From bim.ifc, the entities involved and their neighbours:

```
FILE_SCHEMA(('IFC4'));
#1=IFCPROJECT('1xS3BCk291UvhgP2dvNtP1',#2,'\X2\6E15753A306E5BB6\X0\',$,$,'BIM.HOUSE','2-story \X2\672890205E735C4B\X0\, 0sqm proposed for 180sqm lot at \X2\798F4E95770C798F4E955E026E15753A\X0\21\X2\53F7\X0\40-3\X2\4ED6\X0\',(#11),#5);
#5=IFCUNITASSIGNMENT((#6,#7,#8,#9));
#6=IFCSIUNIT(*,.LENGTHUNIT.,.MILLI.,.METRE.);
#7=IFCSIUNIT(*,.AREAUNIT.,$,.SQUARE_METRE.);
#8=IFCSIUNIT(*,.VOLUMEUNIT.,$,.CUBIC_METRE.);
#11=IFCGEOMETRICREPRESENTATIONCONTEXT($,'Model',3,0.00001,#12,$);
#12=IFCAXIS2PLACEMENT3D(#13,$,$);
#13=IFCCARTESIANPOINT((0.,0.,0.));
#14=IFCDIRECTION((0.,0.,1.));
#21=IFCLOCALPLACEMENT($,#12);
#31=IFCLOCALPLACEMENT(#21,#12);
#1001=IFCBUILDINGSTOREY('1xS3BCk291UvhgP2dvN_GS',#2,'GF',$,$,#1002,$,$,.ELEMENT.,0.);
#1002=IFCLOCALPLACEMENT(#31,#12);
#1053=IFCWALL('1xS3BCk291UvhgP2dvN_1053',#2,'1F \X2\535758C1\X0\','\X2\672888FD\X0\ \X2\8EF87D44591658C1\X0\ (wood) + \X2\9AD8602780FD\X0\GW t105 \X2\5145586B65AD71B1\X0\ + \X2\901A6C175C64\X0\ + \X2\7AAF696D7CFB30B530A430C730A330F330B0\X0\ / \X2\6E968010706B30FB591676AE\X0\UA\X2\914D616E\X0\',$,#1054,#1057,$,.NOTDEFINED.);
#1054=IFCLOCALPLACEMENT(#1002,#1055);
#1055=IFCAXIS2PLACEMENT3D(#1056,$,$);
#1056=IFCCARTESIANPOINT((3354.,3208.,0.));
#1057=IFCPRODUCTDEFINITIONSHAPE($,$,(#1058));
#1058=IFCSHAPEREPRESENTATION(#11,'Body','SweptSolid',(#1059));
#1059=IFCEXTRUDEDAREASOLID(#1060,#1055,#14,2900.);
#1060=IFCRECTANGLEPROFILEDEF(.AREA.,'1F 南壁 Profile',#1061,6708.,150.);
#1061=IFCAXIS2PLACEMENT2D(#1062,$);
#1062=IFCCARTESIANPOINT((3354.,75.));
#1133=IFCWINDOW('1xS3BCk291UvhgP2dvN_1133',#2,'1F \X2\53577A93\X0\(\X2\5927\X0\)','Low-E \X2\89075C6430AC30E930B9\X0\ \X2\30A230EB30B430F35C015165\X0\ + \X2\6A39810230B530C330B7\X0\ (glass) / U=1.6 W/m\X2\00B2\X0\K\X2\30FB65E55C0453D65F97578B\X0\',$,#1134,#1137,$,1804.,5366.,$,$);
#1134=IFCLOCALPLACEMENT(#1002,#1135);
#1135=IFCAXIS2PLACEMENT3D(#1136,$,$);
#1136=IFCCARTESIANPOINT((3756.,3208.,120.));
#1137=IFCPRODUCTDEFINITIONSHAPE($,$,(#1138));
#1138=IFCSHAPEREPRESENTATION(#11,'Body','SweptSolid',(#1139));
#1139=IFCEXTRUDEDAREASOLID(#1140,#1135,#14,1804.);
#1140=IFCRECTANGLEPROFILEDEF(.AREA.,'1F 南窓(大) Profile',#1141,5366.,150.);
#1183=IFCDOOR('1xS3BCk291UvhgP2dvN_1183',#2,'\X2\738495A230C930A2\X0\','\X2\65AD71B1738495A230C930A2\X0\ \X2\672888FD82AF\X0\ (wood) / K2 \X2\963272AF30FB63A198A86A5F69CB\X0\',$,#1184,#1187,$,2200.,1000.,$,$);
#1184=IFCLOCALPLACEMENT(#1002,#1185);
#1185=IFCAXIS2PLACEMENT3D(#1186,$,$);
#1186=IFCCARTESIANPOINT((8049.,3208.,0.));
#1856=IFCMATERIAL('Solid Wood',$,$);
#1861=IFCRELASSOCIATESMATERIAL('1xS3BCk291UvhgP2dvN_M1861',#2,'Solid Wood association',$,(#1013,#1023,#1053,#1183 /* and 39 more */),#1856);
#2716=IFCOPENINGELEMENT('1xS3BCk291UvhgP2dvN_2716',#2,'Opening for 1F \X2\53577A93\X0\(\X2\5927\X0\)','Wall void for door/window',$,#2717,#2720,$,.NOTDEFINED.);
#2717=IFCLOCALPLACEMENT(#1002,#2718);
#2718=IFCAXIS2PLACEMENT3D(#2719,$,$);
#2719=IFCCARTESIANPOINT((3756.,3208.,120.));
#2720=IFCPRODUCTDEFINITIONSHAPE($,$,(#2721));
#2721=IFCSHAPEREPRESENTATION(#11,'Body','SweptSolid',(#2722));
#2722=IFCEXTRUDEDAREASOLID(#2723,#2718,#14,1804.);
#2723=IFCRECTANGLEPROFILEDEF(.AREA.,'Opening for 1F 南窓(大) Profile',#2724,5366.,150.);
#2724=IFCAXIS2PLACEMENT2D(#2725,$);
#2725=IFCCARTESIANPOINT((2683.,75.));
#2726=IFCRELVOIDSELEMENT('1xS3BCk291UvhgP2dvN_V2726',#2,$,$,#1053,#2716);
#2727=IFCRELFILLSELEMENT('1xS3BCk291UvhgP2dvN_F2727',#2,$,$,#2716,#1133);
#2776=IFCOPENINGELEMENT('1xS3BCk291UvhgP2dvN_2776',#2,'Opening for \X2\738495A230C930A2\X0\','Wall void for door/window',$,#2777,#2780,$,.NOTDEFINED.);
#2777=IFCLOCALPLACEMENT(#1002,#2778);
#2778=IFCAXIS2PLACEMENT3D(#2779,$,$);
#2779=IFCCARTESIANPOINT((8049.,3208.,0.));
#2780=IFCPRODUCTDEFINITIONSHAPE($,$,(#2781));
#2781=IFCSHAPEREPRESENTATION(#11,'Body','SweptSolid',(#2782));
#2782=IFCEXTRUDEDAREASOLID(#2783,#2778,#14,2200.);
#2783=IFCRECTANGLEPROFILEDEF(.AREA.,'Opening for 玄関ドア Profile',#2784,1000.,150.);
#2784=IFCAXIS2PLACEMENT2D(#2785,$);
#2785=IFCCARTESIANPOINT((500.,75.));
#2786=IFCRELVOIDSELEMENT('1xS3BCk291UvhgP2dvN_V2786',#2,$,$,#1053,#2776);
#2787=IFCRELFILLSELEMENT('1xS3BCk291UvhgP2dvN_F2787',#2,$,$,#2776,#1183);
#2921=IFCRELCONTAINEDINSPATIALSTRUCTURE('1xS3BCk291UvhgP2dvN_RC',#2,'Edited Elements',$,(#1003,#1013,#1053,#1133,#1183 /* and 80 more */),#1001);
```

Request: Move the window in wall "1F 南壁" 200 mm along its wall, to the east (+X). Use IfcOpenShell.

```python
import ifcopenshell
import ifcopenshell.api.geometry
import ifcopenshell.util.placement
import ifcopenshell.util.unit

model = ifcopenshell.open("bim.ifc")
unit_scale = ifcopenshell.util.unit.calculate_unit_scale(model)

window = model.by_guid("1xS3BCk291UvhgP2dvN_1133")
opening = window.FillsVoids[0].RelatingOpeningElement
wall = opening.VoidsElements[0].RelatingBuildingElement

wall_matrix = ifcopenshell.util.placement.get_local_placement(wall.ObjectPlacement)
shift = wall_matrix[:3, 0] * 0.2 / unit_scale
before = ifcopenshell.util.placement.get_local_placement(window.ObjectPlacement)[:3, 3].copy()

# The window is not placed relative to its opening, so move both.
for product in (opening, window):
    matrix = ifcopenshell.util.placement.get_local_placement(product.ObjectPlacement)
    matrix[:3, 3] += shift
    ifcopenshell.api.geometry.edit_object_placement(model, product=product, matrix=matrix, is_si=False)

after = ifcopenshell.util.placement.get_local_placement(window.ObjectPlacement)[:3, 3]
print("window moved by", (after - before).round(3) + 0.0)

model.write("bim_edited.ifc")
```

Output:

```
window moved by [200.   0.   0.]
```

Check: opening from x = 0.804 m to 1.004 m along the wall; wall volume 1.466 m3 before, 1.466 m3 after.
